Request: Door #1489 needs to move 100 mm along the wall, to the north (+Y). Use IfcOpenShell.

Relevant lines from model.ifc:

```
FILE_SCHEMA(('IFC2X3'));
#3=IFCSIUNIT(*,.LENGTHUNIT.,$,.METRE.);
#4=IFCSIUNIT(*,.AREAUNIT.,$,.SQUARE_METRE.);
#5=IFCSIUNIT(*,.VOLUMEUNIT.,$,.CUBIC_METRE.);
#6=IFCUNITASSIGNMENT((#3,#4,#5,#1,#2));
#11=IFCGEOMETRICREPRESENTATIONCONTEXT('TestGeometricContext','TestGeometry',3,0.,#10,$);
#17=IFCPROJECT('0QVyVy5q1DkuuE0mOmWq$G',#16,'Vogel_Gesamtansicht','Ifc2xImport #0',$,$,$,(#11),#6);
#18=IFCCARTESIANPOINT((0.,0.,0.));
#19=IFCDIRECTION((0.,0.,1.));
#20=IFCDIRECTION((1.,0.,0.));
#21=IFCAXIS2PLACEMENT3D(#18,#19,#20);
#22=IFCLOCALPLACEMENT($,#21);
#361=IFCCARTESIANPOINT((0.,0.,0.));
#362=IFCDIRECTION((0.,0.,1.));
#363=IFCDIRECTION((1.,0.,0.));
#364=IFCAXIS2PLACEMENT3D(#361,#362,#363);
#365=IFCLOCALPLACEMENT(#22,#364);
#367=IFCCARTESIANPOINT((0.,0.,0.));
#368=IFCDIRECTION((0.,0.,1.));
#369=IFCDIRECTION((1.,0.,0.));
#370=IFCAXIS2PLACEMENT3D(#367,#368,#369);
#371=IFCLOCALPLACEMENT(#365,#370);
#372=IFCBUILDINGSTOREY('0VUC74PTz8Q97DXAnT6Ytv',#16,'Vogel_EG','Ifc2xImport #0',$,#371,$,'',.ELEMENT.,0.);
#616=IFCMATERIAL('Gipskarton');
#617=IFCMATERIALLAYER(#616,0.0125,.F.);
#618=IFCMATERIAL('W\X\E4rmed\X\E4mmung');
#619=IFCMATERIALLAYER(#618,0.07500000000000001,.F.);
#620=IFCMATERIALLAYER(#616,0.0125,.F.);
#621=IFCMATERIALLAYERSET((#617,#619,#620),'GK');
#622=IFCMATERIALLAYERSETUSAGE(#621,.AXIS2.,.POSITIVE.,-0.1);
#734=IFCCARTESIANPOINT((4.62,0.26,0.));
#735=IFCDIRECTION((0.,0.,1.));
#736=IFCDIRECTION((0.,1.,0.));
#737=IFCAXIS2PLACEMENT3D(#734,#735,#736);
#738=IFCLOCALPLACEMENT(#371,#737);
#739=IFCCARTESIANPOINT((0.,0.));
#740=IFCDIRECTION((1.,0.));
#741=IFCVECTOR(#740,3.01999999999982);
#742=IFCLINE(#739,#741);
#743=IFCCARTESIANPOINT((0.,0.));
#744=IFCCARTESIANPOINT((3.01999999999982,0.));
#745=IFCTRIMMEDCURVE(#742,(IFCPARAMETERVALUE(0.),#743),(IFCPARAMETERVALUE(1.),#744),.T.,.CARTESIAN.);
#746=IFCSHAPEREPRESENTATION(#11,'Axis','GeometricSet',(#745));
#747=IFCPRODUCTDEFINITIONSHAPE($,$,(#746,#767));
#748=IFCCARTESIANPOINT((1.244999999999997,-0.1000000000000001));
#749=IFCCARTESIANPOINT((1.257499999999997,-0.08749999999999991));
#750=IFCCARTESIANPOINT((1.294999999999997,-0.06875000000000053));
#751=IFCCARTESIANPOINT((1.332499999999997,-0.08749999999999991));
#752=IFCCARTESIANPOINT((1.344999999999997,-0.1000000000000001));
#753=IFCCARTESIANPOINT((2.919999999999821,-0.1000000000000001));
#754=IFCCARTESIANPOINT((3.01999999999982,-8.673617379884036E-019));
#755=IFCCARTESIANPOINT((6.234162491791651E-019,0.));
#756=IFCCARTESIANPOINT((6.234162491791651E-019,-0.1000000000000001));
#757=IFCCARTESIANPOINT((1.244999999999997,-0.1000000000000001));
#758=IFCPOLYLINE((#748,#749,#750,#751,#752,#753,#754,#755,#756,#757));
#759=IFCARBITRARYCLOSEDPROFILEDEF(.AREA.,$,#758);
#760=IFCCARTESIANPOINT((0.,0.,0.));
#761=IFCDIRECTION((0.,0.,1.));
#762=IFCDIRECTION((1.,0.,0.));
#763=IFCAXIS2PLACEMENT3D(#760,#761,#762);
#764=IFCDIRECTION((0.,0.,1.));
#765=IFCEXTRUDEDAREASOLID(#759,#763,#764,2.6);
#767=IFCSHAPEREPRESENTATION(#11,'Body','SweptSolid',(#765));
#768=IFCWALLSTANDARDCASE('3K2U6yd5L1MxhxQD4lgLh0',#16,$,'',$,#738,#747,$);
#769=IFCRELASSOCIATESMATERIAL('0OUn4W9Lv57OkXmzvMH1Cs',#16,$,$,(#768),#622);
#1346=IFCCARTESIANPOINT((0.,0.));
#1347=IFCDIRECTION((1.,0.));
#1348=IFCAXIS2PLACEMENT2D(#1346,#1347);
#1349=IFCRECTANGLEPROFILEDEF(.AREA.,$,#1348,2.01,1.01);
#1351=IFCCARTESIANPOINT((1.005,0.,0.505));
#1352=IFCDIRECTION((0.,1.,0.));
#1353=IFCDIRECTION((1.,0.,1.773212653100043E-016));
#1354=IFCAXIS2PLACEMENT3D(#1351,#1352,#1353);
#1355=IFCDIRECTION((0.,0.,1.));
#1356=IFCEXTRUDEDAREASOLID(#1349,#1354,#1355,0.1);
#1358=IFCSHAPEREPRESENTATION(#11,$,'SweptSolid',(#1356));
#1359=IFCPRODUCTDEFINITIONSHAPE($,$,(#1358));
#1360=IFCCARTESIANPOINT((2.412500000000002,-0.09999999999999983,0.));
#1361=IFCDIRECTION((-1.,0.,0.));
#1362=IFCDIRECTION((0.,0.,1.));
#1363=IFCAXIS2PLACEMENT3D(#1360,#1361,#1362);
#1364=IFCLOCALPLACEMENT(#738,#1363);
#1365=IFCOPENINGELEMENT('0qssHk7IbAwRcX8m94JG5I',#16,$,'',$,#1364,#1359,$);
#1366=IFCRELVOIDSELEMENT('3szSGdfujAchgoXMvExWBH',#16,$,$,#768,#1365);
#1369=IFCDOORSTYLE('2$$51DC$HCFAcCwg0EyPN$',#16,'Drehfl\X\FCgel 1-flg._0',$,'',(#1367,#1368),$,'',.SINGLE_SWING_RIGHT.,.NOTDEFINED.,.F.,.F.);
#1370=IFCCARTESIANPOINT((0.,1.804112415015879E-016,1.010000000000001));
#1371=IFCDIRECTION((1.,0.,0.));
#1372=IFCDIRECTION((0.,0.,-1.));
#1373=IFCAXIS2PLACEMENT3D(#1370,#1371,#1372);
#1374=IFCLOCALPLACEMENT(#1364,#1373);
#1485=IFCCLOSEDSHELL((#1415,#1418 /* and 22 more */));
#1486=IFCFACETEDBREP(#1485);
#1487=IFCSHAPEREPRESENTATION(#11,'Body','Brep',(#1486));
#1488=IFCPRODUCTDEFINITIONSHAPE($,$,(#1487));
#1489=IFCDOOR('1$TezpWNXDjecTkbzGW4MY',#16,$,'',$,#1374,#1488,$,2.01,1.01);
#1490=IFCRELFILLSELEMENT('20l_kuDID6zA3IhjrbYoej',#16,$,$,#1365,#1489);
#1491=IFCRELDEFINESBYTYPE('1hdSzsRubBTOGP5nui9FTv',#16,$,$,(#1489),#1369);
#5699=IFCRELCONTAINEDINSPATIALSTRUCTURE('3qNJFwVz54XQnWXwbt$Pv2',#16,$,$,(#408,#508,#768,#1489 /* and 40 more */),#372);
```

```python
import ifcopenshell
import ifcopenshell.api.geometry
import ifcopenshell.util.placement
import ifcopenshell.util.unit

model = ifcopenshell.open("model.ifc")
unit_scale = ifcopenshell.util.unit.calculate_unit_scale(model)

door = model.by_guid("1$TezpWNXDjecTkbzGW4MY")
opening = door.FillsVoids[0].RelatingOpeningElement
wall = opening.VoidsElements[0].RelatingBuildingElement

wall_matrix = ifcopenshell.util.placement.get_local_placement(wall.ObjectPlacement)
shift = wall_matrix[:3, 0] * 0.1 / unit_scale
before = ifcopenshell.util.placement.get_local_placement(door.ObjectPlacement)[:3, 3].copy()

# The door is placed relative to its opening, so it follows when the opening moves.
matrix = ifcopenshell.util.placement.get_local_placement(opening.ObjectPlacement)
matrix[:3, 3] += shift
ifcopenshell.api.geometry.edit_object_placement(
    model, product=opening, matrix=matrix, is_si=False, should_transform_children=True
)

after = ifcopenshell.util.placement.get_local_placement(door.ObjectPlacement)[:3, 3]
print("door moved by", (after - before).round(3) + 0.0)

model.write("model_v2.ifc")
```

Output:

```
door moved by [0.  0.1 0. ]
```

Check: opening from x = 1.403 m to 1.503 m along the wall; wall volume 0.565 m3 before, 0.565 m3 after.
